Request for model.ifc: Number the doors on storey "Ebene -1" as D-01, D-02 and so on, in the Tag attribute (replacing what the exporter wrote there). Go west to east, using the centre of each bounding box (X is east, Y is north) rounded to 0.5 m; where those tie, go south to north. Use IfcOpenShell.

First a look at what the model holds.

```python
import ifcopenshell
import ifcopenshell.util.element
import ifcopenshell.util.placement

model = ifcopenshell.open("model.ifc")
print(model.schema)
storey = next(s for s in model.by_type("IfcBuildingStorey") if s.Name == "Ebene -1")
doors = [e for e in ifcopenshell.util.element.get_decomposition(storey) if e.is_a("IfcDoor")]
for e in sorted(doors, key=lambda e: e.id()):
    origin = ifcopenshell.util.placement.get_local_placement(e.ObjectPlacement)[:3, 3]
    print(e.id(), e.Tag, e.Name, origin.round(2) + 0.0, sep=" | ")
```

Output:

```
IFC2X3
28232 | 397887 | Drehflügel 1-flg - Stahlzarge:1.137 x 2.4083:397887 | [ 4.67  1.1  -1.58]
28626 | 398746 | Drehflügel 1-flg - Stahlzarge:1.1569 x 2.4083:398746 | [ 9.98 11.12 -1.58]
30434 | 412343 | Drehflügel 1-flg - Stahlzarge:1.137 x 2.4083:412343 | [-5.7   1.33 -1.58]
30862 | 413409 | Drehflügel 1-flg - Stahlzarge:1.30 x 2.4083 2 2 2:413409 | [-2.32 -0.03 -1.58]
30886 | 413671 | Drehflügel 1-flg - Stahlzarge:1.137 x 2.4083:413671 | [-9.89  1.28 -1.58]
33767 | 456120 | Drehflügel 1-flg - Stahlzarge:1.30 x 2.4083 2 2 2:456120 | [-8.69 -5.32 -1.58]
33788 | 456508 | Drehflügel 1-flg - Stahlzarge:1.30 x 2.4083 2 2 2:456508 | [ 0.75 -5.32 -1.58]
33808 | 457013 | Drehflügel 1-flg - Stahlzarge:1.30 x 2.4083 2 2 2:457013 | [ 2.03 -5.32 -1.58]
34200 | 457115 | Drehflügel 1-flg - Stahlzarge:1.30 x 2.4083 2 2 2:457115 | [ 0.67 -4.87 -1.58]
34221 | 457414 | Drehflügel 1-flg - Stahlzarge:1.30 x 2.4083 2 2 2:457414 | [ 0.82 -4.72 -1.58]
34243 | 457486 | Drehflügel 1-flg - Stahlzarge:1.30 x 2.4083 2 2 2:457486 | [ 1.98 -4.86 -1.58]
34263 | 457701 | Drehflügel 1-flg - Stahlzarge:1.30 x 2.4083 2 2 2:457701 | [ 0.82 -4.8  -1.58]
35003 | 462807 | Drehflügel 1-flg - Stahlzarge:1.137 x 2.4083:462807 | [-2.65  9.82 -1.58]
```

```python
import ifcopenshell
import ifcopenshell.geom
import ifcopenshell.util.element
import ifcopenshell.util.shape

model = ifcopenshell.open("model.ifc")
settings = ifcopenshell.geom.settings()
settings.set("use-world-coords", True)


def centre(element):
    shape = ifcopenshell.geom.create_shape(settings, element)
    return ifcopenshell.util.shape.get_bbox_centroid(shape.geometry)


storey = next(s for s in model.by_type("IfcBuildingStorey") if s.Name == "Ebene -1")
doors = [e for e in ifcopenshell.util.element.get_decomposition(storey) if e.is_a("IfcDoor")]

# Insertion points can sit at a corner or the storey origin, so sort by the geometry (in metres).
centres = {e: centre(e) for e in doors}
doors.sort(key=lambda e: (round(centres[e][0] / 0.5), centres[e][1]))

for i, e in enumerate(doors, start=1):
    number = f"D-{i:02d}"
    e.Tag = number
    print(e.id(), number)

model.write("model_edited.ifc")
```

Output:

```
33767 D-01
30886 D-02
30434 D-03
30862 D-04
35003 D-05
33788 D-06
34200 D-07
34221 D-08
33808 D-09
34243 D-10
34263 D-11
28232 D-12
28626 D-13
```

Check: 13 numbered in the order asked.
